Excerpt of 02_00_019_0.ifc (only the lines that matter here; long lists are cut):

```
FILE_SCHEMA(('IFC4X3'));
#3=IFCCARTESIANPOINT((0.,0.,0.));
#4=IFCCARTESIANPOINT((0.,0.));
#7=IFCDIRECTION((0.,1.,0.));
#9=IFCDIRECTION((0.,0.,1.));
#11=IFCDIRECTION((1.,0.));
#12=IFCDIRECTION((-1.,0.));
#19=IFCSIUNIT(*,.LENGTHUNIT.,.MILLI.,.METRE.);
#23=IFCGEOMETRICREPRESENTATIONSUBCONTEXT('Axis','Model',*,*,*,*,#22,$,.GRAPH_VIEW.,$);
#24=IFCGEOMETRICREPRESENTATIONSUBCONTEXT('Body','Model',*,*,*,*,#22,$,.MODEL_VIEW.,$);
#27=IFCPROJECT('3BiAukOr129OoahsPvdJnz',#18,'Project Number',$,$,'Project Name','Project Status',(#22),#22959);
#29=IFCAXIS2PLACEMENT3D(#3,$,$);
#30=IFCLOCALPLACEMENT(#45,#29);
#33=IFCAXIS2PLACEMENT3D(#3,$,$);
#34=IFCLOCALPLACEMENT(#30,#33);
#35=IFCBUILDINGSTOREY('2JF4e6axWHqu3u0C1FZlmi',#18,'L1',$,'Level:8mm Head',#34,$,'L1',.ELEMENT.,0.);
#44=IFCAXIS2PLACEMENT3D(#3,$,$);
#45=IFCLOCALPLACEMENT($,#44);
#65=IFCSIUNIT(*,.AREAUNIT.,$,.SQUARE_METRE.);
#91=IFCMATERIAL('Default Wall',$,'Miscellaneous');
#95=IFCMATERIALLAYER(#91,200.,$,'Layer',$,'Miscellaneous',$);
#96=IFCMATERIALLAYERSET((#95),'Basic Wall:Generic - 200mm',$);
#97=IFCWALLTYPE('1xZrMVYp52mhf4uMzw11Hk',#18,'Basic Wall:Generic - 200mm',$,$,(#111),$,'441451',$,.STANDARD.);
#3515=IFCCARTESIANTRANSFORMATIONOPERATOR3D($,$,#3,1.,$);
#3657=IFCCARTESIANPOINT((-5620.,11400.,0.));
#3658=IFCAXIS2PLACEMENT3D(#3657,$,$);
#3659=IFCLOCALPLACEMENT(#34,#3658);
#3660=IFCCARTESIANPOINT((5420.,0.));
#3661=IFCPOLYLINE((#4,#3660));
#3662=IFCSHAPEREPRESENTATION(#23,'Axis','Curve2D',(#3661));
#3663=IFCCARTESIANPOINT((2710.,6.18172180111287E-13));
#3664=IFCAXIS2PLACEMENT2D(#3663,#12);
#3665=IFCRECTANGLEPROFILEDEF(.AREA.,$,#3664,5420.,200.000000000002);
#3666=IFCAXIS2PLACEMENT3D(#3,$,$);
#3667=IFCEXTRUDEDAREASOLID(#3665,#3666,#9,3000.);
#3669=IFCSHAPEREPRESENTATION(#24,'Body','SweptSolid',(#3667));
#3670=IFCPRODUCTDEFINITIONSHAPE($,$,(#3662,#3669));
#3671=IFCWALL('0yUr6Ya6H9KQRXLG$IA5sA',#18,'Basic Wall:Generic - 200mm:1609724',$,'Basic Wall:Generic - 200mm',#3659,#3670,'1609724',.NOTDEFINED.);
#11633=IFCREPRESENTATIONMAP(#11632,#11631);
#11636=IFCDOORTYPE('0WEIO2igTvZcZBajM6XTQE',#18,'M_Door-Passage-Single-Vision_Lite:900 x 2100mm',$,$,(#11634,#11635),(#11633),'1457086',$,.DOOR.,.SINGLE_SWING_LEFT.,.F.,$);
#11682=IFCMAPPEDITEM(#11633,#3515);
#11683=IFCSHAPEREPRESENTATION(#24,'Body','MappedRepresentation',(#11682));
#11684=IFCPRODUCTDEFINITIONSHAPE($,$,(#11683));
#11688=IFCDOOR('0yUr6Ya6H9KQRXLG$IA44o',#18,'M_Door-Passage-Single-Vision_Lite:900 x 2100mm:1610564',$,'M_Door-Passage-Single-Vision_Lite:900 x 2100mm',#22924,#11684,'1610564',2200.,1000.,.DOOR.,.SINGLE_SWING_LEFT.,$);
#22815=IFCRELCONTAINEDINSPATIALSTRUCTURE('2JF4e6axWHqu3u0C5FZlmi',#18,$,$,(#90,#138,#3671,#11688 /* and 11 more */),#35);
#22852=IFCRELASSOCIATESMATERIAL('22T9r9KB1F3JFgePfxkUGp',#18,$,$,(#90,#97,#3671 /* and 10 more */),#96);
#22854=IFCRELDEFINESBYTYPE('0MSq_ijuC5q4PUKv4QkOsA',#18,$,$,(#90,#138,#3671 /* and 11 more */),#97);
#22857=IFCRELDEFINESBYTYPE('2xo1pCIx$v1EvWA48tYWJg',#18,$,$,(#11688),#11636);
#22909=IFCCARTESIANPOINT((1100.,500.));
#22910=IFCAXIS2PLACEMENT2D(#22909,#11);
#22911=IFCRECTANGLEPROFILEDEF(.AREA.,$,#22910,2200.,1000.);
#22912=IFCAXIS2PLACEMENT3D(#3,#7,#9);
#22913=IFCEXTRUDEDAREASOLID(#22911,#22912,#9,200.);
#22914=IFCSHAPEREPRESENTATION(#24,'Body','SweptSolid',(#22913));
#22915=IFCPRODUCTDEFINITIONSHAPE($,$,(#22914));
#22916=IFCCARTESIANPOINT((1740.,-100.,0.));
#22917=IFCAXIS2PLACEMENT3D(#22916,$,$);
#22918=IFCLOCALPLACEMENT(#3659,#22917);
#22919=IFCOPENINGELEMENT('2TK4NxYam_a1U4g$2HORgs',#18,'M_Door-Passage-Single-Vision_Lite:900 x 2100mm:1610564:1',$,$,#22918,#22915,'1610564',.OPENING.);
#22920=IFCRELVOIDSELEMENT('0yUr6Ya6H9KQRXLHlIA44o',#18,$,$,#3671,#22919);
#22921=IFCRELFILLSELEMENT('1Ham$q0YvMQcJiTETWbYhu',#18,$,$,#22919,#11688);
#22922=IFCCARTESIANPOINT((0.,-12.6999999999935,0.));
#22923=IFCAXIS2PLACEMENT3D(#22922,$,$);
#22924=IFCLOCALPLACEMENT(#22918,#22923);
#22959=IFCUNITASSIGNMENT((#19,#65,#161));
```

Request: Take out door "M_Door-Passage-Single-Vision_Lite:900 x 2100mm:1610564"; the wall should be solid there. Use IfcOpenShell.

```python
import ifcopenshell
import ifcopenshell.api.feature
import ifcopenshell.api.root
import ifcopenshell.geom
import ifcopenshell.util.shape

model = ifcopenshell.open("02_00_019_0.ifc")
settings = ifcopenshell.geom.settings()


def volume(element):
    """Net volume in cubic metres, openings subtracted."""
    shape = ifcopenshell.geom.create_shape(settings, element)
    return ifcopenshell.util.shape.get_volume(shape.geometry)


door = model.by_guid("0yUr6Ya6H9KQRXLG$IA44o")
opening = door.FillsVoids[0].RelatingOpeningElement
wall = opening.VoidsElements[0].RelatingBuildingElement
before = volume(wall)

ifcopenshell.api.root.remove_product(model, product=door)
ifcopenshell.api.feature.remove_feature(model, feature=opening)

after = volume(wall)

print(f"wall volume {before:.3f} -> {after:.3f} m3")

model.write("02_00_019_0_updated.ifc")
```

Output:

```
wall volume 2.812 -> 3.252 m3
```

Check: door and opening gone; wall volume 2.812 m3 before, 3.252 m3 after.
